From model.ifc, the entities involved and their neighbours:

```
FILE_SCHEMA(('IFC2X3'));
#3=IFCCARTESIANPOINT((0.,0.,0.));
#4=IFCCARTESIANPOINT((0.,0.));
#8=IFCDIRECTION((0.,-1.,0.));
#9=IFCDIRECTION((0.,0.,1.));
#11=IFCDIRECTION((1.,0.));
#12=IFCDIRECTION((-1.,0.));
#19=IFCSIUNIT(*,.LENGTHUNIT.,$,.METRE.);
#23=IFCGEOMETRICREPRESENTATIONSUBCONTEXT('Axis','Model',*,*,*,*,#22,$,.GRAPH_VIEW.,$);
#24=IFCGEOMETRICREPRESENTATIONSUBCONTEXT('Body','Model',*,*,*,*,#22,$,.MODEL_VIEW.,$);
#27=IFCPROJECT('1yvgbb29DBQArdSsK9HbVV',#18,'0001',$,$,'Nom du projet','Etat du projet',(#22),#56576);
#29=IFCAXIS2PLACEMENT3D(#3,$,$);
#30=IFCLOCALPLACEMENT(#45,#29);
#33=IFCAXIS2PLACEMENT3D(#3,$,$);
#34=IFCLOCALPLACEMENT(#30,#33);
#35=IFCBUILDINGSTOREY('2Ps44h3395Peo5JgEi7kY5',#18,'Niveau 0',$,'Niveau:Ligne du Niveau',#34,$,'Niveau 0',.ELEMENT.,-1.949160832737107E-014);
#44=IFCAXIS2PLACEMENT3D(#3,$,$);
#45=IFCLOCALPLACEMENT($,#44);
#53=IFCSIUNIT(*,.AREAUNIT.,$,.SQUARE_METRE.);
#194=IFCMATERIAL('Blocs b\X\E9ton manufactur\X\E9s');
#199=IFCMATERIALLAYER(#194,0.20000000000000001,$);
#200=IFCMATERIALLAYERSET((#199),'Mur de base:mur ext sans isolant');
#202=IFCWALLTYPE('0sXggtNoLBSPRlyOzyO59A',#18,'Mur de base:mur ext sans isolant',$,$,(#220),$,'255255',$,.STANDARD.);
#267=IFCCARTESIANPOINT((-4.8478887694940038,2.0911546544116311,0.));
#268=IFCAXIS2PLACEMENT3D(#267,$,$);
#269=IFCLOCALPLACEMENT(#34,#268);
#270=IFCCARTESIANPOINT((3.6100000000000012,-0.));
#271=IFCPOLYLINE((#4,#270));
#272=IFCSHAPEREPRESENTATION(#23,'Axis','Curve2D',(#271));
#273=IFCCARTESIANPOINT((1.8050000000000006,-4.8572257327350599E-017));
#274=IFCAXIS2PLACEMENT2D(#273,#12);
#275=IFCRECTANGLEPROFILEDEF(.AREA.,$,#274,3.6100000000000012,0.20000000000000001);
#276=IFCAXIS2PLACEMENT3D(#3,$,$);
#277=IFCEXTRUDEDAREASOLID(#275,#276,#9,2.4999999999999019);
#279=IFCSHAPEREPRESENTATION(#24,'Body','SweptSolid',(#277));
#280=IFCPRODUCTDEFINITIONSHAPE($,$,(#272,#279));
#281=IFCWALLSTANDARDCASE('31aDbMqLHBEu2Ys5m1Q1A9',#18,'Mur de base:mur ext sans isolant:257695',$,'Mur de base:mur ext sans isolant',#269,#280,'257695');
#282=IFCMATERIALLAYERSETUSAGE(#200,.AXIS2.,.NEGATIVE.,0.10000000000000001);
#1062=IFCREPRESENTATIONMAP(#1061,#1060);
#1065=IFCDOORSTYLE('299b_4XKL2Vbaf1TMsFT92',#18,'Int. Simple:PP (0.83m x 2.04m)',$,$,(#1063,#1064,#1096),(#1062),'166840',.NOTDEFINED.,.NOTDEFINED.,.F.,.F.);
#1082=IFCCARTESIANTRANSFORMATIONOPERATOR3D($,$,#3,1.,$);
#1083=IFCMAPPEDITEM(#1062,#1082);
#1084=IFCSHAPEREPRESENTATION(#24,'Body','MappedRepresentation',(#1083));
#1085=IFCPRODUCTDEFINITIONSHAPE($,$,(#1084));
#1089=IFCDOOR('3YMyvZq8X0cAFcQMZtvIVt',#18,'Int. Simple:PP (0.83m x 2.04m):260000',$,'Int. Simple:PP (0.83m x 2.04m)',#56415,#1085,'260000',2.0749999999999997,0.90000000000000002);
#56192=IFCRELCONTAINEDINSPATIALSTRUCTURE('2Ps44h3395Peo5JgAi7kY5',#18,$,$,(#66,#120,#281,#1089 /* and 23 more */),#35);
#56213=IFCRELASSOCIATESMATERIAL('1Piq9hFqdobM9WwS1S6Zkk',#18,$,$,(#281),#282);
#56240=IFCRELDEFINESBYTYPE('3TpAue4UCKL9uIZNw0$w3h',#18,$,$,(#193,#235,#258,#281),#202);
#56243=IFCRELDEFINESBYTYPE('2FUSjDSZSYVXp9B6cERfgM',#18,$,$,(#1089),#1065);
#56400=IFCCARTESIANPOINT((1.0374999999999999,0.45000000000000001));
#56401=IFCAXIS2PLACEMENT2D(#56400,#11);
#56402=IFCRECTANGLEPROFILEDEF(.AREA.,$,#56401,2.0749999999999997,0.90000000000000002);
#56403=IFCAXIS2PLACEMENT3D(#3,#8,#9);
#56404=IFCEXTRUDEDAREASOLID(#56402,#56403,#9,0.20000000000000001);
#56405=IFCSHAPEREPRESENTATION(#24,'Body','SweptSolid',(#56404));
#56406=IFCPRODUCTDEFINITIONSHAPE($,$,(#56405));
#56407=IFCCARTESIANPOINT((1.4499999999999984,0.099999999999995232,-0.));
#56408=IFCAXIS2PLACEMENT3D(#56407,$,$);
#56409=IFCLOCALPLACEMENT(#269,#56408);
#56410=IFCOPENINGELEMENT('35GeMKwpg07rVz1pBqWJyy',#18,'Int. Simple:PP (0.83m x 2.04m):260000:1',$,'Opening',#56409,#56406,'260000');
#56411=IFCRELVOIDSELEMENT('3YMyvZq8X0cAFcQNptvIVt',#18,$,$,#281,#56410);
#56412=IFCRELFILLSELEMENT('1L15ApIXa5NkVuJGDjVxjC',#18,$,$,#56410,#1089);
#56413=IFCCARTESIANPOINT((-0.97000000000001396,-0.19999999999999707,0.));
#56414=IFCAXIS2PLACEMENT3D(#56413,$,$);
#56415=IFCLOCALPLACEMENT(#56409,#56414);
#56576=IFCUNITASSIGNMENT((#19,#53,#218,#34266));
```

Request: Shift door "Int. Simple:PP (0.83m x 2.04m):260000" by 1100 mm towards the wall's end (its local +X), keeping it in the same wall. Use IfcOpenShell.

```python
import ifcopenshell
import ifcopenshell.api.geometry
import ifcopenshell.util.placement

model = ifcopenshell.open("model.ifc")

door = model.by_id(1089)
opening = door.FillsVoids[0].RelatingOpeningElement
wall = opening.VoidsElements[0].RelatingBuildingElement

wall_matrix = ifcopenshell.util.placement.get_local_placement(wall.ObjectPlacement)
shift = wall_matrix[:3, 0] * 1.1
before = ifcopenshell.util.placement.get_local_placement(door.ObjectPlacement)[:3, 3].copy()

# The door is placed relative to its opening, so it follows when the opening moves.
matrix = ifcopenshell.util.placement.get_local_placement(opening.ObjectPlacement)
matrix[:3, 3] += shift
ifcopenshell.api.geometry.edit_object_placement(
    model, product=opening, matrix=matrix, is_si=False, should_transform_children=True
)

after = ifcopenshell.util.placement.get_local_placement(door.ObjectPlacement)[:3, 3]
print("door moved by", (after - before).round(3) + 0.0)

model.write("model_edited.ifc")
```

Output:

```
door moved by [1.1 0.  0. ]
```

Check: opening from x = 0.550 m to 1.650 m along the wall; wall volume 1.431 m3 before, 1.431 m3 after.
